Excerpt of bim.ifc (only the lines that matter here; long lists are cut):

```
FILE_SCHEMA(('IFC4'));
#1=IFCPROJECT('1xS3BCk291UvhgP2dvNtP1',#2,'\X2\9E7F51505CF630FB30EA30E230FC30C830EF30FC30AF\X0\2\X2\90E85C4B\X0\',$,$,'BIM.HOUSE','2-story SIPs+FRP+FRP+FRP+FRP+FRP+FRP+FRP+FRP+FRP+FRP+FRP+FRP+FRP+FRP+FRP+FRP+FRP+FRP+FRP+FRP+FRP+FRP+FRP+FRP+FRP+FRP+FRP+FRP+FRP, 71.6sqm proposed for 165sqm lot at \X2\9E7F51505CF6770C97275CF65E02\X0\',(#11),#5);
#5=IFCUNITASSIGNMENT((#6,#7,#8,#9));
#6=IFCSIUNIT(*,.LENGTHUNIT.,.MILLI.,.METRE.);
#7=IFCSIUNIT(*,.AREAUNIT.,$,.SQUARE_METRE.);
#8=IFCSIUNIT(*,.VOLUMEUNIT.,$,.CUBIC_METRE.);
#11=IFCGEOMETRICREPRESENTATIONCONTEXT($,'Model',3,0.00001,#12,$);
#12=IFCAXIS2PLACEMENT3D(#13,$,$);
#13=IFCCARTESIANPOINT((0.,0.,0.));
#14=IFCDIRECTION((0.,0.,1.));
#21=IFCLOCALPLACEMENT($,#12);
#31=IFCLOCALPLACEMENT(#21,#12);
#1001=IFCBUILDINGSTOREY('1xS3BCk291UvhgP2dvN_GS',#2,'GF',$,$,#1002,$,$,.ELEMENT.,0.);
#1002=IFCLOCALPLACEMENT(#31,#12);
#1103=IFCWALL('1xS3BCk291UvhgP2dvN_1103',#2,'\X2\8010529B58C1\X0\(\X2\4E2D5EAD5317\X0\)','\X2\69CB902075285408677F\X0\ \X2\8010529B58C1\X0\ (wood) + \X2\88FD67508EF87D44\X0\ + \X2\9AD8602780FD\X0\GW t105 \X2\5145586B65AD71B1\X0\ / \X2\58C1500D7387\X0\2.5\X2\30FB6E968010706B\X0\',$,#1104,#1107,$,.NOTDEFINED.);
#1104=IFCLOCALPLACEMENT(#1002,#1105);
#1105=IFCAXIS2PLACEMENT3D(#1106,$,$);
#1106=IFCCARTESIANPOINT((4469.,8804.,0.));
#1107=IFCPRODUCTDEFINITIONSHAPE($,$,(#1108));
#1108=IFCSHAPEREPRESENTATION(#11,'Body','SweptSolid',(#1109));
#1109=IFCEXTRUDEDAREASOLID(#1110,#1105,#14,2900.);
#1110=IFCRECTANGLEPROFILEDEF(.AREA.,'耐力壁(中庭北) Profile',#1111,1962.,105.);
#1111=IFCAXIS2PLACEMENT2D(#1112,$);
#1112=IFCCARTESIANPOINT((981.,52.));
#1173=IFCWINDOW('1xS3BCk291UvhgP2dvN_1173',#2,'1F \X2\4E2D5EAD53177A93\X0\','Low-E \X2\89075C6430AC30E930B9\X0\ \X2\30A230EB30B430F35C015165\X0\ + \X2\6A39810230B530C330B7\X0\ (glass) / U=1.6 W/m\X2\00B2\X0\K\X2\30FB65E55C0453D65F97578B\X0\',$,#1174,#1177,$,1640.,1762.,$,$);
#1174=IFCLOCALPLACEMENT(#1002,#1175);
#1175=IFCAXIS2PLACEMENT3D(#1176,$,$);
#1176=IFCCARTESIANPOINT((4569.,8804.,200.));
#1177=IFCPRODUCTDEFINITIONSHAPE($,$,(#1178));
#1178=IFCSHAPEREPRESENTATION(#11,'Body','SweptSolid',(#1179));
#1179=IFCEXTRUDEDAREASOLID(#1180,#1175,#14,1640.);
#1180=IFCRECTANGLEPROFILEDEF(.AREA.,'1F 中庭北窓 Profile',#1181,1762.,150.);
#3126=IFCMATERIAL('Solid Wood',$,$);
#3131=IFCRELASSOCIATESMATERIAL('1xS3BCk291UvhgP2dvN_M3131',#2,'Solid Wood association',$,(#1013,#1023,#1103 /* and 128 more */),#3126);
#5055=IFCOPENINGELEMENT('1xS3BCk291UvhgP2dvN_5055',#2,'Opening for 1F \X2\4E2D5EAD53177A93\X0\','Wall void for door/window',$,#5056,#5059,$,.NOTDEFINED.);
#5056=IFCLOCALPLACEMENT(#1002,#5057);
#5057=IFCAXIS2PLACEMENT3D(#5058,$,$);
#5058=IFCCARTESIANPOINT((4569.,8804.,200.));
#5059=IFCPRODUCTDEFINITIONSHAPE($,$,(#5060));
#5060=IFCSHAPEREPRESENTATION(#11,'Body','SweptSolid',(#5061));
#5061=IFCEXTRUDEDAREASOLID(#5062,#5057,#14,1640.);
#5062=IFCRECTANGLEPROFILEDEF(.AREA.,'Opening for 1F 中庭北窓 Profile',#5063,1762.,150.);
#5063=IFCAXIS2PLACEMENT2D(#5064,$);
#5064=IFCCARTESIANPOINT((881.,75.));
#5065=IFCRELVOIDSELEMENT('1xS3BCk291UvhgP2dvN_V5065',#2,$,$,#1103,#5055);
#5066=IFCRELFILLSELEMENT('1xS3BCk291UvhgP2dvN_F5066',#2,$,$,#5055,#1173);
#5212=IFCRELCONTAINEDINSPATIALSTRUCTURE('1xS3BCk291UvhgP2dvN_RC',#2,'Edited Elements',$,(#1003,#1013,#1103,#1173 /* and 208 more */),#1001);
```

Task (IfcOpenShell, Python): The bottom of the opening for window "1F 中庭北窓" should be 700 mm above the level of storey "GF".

```python
import numpy as np
import ifcopenshell
import ifcopenshell.api.geometry
import ifcopenshell.geom
import ifcopenshell.util.element
import ifcopenshell.util.placement
import ifcopenshell.util.shape
import ifcopenshell.util.unit

model = ifcopenshell.open("bim.ifc")
unit_scale = ifcopenshell.util.unit.calculate_unit_scale(model)

window = model.by_guid("1xS3BCk291UvhgP2dvN_1173")
opening = window.FillsVoids[0].RelatingOpeningElement
storey = ifcopenshell.util.element.get_container(window, ifc_class="IfcBuildingStorey")
level = ifcopenshell.util.placement.get_local_placement(storey.ObjectPlacement)[2, 3]

# The opening's origin need not be at the sill, so measure its lowest point.
shape = ifcopenshell.geom.create_shape(ifcopenshell.geom.settings(), opening)
bottom = ifcopenshell.util.shape.get_shape_bottom_elevation(shape, shape.geometry) / unit_scale
dz = level + 700.0 - bottom

shift = np.array([0.0, 0.0, dz])
# The window is not placed relative to its opening, so move both.
for product in (opening, window):
    matrix = ifcopenshell.util.placement.get_local_placement(product.ObjectPlacement)
    matrix[:3, 3] += shift
    ifcopenshell.api.geometry.edit_object_placement(model, product=product, matrix=matrix, is_si=False)

print(f"moved by {dz * unit_scale:+.3f} m")

model.write("bim_v2.ifc")
```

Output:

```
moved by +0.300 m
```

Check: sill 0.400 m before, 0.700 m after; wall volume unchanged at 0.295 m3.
